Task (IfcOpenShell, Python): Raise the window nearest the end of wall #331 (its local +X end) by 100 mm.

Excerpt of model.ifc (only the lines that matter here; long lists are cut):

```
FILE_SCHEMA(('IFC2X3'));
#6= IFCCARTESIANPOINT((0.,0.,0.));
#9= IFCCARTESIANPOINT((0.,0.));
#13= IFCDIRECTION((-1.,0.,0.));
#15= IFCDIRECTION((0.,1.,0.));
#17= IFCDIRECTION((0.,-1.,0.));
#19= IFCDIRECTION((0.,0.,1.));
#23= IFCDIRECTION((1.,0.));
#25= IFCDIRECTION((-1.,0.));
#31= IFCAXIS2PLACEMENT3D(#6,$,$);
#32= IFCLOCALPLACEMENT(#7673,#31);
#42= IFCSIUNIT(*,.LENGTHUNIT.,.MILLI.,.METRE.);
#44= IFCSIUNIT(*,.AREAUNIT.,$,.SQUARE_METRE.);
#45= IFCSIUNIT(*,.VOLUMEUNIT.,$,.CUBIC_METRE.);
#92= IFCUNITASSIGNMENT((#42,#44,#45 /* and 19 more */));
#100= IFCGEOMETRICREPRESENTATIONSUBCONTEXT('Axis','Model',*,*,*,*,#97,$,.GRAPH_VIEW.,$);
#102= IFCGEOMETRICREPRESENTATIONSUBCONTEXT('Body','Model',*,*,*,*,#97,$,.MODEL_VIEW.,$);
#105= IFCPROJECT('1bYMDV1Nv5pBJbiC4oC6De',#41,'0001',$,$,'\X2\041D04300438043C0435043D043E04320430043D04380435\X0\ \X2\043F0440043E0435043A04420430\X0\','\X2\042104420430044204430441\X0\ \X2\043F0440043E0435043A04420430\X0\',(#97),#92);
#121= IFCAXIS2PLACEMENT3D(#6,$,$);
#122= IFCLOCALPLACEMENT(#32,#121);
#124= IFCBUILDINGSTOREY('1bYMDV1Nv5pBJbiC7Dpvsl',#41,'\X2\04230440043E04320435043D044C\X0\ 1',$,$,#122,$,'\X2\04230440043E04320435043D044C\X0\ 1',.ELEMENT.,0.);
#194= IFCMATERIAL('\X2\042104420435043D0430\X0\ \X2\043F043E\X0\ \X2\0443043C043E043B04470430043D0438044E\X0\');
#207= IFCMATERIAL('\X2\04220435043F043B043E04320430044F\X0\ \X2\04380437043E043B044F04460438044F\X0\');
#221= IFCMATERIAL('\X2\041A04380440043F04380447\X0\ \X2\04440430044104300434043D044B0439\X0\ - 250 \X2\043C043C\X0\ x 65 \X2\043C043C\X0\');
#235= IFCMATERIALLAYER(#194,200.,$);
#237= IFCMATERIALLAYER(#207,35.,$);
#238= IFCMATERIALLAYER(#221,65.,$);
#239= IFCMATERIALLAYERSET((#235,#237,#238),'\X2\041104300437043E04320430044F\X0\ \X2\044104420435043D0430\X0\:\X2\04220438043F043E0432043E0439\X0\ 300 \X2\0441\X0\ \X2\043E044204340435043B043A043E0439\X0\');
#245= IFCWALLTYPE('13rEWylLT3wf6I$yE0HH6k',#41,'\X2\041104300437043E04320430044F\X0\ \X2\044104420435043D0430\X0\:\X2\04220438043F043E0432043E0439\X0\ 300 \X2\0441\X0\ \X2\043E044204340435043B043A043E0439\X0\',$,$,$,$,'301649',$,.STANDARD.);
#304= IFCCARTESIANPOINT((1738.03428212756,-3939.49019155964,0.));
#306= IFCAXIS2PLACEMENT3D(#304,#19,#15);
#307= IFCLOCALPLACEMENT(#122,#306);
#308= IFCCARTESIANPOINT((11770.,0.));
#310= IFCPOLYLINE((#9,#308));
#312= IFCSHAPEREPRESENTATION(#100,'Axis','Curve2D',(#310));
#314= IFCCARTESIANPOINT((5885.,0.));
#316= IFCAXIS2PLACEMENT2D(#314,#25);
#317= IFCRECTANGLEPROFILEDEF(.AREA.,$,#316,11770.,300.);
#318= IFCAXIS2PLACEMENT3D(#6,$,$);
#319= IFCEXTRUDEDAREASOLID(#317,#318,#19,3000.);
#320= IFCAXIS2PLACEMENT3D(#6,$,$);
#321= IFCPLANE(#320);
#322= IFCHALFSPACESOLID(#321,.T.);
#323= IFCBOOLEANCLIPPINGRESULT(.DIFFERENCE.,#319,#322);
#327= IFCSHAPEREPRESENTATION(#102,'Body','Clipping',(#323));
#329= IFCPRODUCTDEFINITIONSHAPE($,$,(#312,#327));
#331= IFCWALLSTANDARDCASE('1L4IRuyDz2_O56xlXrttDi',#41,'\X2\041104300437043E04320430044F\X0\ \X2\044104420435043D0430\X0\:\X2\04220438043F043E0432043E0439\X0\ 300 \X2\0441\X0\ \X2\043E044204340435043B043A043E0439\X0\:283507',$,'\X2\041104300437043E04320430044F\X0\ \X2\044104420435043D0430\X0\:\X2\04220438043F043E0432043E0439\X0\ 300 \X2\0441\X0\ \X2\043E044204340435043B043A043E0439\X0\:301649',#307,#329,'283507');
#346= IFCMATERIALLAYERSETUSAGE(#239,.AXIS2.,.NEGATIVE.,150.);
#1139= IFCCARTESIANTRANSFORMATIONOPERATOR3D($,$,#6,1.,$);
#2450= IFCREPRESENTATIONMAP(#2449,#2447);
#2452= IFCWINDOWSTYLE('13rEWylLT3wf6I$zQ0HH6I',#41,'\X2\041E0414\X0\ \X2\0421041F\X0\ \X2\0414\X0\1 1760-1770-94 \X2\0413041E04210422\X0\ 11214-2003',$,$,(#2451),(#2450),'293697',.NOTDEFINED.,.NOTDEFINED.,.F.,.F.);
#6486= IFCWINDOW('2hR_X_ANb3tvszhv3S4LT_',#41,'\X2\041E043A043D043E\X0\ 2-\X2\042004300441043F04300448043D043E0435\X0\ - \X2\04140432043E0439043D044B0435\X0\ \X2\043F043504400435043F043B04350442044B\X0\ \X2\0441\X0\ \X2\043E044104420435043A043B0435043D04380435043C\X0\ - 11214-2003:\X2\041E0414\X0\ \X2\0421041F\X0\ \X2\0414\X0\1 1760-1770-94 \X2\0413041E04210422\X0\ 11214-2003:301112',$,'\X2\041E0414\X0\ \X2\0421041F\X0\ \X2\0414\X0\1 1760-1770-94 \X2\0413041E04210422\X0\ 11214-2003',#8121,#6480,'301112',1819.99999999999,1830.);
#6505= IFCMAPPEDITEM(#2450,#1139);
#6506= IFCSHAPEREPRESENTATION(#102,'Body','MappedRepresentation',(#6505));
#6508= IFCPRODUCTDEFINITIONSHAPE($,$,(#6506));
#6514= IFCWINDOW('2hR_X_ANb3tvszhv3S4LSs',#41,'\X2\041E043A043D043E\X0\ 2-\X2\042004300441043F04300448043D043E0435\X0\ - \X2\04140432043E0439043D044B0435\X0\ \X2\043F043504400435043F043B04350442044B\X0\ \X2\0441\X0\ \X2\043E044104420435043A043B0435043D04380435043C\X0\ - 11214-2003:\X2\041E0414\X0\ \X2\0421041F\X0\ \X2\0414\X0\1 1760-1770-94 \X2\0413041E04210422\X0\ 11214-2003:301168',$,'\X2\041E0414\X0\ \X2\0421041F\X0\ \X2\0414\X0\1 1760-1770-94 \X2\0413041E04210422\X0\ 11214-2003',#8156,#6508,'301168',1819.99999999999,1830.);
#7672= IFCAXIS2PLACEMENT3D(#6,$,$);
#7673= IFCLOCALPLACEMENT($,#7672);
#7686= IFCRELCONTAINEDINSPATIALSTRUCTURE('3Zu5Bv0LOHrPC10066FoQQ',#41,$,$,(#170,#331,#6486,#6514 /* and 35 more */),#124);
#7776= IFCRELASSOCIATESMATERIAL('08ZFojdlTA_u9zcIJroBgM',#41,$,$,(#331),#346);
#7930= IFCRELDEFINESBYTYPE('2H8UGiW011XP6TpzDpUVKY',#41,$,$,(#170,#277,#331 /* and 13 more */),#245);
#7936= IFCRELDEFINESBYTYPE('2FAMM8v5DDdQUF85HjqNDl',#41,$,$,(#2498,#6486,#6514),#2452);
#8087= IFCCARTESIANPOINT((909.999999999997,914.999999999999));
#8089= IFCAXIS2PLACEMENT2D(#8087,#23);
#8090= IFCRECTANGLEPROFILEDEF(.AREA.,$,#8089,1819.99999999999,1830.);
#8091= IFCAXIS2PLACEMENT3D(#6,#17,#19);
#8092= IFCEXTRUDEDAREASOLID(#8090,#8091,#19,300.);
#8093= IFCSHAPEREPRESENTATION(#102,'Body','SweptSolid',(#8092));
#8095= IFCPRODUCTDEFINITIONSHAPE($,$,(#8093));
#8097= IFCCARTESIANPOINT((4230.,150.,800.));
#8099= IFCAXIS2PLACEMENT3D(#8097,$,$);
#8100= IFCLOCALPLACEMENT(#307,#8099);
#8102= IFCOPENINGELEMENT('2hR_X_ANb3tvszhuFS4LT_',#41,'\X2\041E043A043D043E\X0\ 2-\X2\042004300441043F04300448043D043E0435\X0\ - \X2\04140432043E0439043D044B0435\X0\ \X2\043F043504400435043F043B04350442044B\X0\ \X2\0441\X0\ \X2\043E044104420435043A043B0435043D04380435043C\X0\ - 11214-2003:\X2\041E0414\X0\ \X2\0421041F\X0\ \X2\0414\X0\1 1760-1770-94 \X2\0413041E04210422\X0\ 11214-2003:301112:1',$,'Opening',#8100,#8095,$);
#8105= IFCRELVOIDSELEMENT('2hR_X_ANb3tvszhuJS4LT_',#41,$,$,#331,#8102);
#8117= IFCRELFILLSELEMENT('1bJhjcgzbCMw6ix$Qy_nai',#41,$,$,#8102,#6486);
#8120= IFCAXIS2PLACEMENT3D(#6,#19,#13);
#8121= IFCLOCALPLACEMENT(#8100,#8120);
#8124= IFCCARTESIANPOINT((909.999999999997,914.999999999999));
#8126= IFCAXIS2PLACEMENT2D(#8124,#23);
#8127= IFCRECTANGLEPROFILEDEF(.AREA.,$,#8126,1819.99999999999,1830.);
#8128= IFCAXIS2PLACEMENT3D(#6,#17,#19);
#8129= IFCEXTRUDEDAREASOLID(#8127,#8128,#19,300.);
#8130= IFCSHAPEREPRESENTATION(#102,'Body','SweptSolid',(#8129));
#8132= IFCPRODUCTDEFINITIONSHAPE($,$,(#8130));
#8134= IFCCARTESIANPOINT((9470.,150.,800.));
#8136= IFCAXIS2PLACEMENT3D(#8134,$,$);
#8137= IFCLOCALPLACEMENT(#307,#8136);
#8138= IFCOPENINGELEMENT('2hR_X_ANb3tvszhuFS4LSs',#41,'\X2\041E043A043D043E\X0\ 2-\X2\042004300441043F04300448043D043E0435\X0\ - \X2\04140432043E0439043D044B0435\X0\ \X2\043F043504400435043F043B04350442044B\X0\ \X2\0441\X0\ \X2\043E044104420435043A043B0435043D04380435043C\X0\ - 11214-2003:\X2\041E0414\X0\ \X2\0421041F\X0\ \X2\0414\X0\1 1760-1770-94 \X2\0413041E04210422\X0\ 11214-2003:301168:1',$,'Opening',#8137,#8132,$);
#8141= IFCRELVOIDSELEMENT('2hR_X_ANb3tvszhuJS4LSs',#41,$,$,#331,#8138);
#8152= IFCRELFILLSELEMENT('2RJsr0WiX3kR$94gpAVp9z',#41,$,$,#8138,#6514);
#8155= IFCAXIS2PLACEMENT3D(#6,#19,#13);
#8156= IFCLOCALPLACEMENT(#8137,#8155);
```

```python
import numpy as np
import ifcopenshell
import ifcopenshell.api.geometry
import ifcopenshell.util.placement
import ifcopenshell.util.unit

model = ifcopenshell.open("model.ifc")
unit_scale = ifcopenshell.util.unit.calculate_unit_scale(model)

window = model.by_id(6514)
opening = window.FillsVoids[0].RelatingOpeningElement
dz = 100.0

shift = np.array([0.0, 0.0, dz])
# The window is placed relative to its opening, so it follows when the opening moves.
matrix = ifcopenshell.util.placement.get_local_placement(opening.ObjectPlacement)
matrix[:3, 3] += shift
ifcopenshell.api.geometry.edit_object_placement(
    model, product=opening, matrix=matrix, is_si=False, should_transform_children=True
)

print(f"moved by {dz * unit_scale:+.3f} m")

model.write("model_updated.ifc")
```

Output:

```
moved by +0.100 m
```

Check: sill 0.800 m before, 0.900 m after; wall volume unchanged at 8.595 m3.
